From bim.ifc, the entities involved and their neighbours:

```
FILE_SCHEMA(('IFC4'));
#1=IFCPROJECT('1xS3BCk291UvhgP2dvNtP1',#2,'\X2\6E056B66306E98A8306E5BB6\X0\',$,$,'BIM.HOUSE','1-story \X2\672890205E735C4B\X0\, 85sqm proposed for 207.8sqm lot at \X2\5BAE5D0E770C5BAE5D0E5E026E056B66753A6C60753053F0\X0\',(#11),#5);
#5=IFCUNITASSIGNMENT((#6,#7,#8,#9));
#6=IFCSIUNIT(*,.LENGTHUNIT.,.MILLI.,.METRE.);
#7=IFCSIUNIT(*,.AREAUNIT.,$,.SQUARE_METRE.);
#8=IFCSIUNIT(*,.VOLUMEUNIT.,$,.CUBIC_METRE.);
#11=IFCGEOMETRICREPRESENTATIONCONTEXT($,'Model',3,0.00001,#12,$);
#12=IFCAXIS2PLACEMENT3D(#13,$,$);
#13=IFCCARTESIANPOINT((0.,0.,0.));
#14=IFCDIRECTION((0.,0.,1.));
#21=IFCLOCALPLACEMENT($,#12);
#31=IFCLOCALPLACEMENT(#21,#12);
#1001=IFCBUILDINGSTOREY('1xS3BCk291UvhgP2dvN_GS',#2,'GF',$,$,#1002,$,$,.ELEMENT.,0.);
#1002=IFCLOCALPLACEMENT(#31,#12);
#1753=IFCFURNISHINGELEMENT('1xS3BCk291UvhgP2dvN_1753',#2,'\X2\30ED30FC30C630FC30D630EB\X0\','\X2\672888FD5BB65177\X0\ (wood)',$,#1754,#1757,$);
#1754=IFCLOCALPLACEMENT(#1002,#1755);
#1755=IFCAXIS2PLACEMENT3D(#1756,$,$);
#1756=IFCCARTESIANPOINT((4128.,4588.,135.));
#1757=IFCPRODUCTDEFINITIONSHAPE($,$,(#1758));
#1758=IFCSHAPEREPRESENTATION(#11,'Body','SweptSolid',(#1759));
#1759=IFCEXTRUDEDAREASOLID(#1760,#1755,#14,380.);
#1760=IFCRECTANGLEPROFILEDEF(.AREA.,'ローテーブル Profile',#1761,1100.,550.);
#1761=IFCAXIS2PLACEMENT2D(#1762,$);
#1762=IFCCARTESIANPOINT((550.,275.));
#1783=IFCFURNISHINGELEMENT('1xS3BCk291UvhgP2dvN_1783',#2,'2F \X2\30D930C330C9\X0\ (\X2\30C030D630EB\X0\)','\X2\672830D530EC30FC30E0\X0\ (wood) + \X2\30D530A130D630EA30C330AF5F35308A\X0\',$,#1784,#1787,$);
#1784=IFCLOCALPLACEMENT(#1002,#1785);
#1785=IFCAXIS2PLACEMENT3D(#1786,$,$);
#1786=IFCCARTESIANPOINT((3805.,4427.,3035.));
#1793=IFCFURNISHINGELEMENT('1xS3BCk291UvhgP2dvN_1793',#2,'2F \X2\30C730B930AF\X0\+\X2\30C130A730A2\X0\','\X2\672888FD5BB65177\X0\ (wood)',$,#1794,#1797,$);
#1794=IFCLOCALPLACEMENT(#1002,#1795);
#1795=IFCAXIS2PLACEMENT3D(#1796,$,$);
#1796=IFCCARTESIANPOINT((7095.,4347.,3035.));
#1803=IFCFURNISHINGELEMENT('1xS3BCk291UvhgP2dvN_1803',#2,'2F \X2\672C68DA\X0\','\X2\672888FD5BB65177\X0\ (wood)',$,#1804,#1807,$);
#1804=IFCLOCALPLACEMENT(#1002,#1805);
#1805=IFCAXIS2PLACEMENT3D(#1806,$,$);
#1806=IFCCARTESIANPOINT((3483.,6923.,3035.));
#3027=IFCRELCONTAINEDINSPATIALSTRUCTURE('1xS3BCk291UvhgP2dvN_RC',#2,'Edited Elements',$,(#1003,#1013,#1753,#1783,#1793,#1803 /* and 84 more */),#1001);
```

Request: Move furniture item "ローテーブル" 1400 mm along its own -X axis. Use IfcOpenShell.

```python
import ifcopenshell
import ifcopenshell.api.geometry
import ifcopenshell.util.placement
import ifcopenshell.util.unit

model = ifcopenshell.open("bim.ifc")
unit_scale = ifcopenshell.util.unit.calculate_unit_scale(model)

item = model.by_guid("1xS3BCk291UvhgP2dvN_1753")
matrix = ifcopenshell.util.placement.get_local_placement(item.ObjectPlacement)
matrix[:3, 3] -= matrix[:3, 0] * 1.4 / unit_scale
ifcopenshell.api.geometry.edit_object_placement(model, product=item, matrix=matrix, is_si=False)

print(ifcopenshell.util.placement.get_local_placement(item.ObjectPlacement).round(3) + 0.0)

model.write("bim_v2.ifc")
```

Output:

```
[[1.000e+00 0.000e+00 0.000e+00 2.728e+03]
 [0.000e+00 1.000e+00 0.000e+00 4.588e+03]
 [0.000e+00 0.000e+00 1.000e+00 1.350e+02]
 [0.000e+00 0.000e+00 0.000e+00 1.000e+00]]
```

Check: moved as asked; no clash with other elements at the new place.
